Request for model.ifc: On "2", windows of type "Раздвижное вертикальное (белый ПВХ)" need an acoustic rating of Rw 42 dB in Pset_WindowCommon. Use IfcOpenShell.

First a look at what the model holds.

```python
import ifcopenshell
import ifcopenshell.util.element

model = ifcopenshell.open("model.ifc")
print(model.schema)
storey = next(s for s in model.by_type("IfcBuildingStorey") if s.Name == "2")
windows = [e for e in ifcopenshell.util.element.get_decomposition(storey) if e.is_a("IfcWindow")]
seen = {}
for e in windows:
    element_type = ifcopenshell.util.element.get_type(e)
    key = (element_type.Name if element_type != e and element_type else None, ifcopenshell.util.element.get_pset(e, "Pset_WindowCommon", "AcousticRating"))
    seen[key] = seen.get(key, 0) + 1
for (name, value), count in sorted(seen.items(), key=str):
    print(count, "x", name, "|", value)
```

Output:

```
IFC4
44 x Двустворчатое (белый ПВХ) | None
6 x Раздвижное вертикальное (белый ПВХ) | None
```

```python
import ifcopenshell
import ifcopenshell.api.pset
import ifcopenshell.util.element

model = ifcopenshell.open("model.ifc")

storey = next(s for s in model.by_type("IfcBuildingStorey") if s.Name == "2")
windows = [e for e in ifcopenshell.util.element.get_decomposition(storey) if e.is_a("IfcWindow")]

count = 0
for e in windows:
    element_type = ifcopenshell.util.element.get_type(e)
    if element_type in (None, e) or element_type.Name != "Раздвижное вертикальное (белый ПВХ)":
        continue
    # add_pset returns the element's existing set when there is one.
    pset = ifcopenshell.api.pset.add_pset(model, product=e, name="Pset_WindowCommon")
    ifcopenshell.api.pset.edit_pset(model, pset=pset, properties={"AcousticRating": "Rw 42 dB"})
    count += 1

print(count, "windows updated")

model.write("model-out.ifc")
```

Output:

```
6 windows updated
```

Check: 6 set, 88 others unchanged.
